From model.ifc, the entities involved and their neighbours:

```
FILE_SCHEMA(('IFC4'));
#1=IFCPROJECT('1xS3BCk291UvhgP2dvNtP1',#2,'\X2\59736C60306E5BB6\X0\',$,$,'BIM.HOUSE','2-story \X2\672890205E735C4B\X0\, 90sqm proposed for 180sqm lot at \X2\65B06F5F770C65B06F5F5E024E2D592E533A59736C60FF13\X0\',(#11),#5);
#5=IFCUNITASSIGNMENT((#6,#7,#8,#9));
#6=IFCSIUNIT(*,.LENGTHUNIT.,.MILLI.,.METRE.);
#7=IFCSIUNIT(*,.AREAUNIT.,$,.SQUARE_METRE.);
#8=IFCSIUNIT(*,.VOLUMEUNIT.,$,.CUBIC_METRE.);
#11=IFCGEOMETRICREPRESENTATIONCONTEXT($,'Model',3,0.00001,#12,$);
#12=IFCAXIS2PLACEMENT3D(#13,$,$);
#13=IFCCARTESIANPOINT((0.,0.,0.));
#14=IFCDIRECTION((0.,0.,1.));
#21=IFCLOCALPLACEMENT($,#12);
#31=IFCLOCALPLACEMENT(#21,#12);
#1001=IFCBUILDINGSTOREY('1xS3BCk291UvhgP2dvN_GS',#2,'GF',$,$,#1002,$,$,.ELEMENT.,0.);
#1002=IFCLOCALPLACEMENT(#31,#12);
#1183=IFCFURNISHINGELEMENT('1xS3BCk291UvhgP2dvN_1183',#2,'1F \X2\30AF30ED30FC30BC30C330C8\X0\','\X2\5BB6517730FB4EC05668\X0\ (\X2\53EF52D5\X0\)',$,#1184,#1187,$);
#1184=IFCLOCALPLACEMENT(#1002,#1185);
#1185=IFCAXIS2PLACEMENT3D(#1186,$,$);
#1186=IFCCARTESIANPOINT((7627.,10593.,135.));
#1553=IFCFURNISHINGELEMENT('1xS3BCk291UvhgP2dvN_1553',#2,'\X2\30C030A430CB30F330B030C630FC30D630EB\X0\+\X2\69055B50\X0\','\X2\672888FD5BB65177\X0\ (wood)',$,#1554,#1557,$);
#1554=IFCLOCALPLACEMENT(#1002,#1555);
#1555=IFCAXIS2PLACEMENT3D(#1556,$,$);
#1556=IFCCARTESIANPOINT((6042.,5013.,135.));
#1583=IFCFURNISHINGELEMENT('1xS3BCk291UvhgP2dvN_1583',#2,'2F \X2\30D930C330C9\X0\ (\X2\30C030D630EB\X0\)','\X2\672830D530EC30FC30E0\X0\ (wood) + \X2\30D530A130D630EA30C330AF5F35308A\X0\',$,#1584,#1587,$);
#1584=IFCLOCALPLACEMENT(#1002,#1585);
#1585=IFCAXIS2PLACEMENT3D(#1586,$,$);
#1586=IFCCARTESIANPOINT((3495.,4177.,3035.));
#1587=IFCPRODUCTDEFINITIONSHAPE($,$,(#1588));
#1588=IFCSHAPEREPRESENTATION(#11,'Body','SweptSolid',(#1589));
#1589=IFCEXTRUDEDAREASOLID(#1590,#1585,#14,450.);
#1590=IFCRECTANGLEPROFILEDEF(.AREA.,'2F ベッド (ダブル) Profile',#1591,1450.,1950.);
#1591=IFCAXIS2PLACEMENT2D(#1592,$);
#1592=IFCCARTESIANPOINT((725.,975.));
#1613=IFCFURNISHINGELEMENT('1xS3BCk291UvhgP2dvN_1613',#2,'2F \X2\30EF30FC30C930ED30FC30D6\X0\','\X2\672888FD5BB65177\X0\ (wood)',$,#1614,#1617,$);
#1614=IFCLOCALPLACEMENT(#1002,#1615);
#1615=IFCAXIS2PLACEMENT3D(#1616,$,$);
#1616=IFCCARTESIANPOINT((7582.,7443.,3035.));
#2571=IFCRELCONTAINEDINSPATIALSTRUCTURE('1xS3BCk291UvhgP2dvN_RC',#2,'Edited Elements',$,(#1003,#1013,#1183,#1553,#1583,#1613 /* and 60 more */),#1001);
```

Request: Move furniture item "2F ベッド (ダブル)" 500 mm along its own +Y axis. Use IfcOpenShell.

```python
import ifcopenshell
import ifcopenshell.api.geometry
import ifcopenshell.util.placement
import ifcopenshell.util.unit

model = ifcopenshell.open("model.ifc")
unit_scale = ifcopenshell.util.unit.calculate_unit_scale(model)

item = model.by_id(1583)
matrix = ifcopenshell.util.placement.get_local_placement(item.ObjectPlacement)
matrix[:3, 3] += matrix[:3, 1] * 0.5 / unit_scale
ifcopenshell.api.geometry.edit_object_placement(model, product=item, matrix=matrix, is_si=False)

print(ifcopenshell.util.placement.get_local_placement(item.ObjectPlacement).round(3) + 0.0)

model.write("model_v2.ifc")
```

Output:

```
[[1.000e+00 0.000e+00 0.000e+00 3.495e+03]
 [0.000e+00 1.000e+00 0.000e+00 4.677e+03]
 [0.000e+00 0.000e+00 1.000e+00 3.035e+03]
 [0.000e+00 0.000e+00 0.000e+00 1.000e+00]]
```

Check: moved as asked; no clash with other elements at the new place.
